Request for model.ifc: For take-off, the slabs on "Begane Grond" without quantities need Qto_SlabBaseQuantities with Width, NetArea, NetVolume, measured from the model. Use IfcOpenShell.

First a look at what the model holds.

```python
import ifcopenshell
import ifcopenshell.util.element
import ifcopenshell.util.unit

model = ifcopenshell.open("model.ifc")
print(model.schema)
for unit_type in ("LENGTHUNIT", "AREAUNIT", "VOLUMEUNIT"):
    print(unit_type, ifcopenshell.util.unit.calculate_unit_scale(model, unit_type))
storey = next(s for s in model.by_type("IfcBuildingStorey") if s.Name == "Begane Grond")
slabs = [e for e in ifcopenshell.util.element.get_decomposition(storey) if e.is_a("IfcSlab")]
for e in sorted(slabs, key=lambda e: e.id()):
    print(e.id(), e.is_a(), e.Name, list(ifcopenshell.util.element.get_psets(e, qtos_only=True)), sep=" | ")
```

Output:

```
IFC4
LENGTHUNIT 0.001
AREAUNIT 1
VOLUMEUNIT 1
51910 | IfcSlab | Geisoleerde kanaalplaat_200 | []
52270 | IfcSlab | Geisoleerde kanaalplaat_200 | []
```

```python
import ifcopenshell
import ifcopenshell.api.pset
import ifcopenshell.geom
import ifcopenshell.util.element
import ifcopenshell.util.shape
import ifcopenshell.util.unit

model = ifcopenshell.open("model.ifc")
unit_scale = ifcopenshell.util.unit.calculate_unit_scale(model)
area_scale = ifcopenshell.util.unit.calculate_unit_scale(model, "AREAUNIT")
volume_scale = ifcopenshell.util.unit.calculate_unit_scale(model, "VOLUMEUNIT")
settings = ifcopenshell.geom.settings()

storey = next(s for s in model.by_type("IfcBuildingStorey") if s.Name == "Begane Grond")
slabs = [e for e in ifcopenshell.util.element.get_decomposition(storey) if e.is_a("IfcSlab")]

for e in sorted(slabs, key=lambda e: e.id()):
    if ifcopenshell.util.element.get_psets(e, qtos_only=True, should_inherit=False):
        continue
    # Geometry comes back in metres, in the element's own axes.
    shape = ifcopenshell.geom.create_shape(settings, e)
    values = {
        "Width": ifcopenshell.util.shape.get_z(shape.geometry) / unit_scale,
        "NetArea": ifcopenshell.util.shape.get_footprint_area(shape.geometry) / area_scale,
        "NetVolume": ifcopenshell.util.shape.get_volume(shape.geometry) / volume_scale,
    }
    qto = ifcopenshell.api.pset.add_qto(model, product=e, name="Qto_SlabBaseQuantities")
    ifcopenshell.api.pset.edit_qto(model, qto=qto, properties=values)
    print(e.id(), {k: round(v, 3) for k, v in values.items()})

model.write("model-out.ifc")
```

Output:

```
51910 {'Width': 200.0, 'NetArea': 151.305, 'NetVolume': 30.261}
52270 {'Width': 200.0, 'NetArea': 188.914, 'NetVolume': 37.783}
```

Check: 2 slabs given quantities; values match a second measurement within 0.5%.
